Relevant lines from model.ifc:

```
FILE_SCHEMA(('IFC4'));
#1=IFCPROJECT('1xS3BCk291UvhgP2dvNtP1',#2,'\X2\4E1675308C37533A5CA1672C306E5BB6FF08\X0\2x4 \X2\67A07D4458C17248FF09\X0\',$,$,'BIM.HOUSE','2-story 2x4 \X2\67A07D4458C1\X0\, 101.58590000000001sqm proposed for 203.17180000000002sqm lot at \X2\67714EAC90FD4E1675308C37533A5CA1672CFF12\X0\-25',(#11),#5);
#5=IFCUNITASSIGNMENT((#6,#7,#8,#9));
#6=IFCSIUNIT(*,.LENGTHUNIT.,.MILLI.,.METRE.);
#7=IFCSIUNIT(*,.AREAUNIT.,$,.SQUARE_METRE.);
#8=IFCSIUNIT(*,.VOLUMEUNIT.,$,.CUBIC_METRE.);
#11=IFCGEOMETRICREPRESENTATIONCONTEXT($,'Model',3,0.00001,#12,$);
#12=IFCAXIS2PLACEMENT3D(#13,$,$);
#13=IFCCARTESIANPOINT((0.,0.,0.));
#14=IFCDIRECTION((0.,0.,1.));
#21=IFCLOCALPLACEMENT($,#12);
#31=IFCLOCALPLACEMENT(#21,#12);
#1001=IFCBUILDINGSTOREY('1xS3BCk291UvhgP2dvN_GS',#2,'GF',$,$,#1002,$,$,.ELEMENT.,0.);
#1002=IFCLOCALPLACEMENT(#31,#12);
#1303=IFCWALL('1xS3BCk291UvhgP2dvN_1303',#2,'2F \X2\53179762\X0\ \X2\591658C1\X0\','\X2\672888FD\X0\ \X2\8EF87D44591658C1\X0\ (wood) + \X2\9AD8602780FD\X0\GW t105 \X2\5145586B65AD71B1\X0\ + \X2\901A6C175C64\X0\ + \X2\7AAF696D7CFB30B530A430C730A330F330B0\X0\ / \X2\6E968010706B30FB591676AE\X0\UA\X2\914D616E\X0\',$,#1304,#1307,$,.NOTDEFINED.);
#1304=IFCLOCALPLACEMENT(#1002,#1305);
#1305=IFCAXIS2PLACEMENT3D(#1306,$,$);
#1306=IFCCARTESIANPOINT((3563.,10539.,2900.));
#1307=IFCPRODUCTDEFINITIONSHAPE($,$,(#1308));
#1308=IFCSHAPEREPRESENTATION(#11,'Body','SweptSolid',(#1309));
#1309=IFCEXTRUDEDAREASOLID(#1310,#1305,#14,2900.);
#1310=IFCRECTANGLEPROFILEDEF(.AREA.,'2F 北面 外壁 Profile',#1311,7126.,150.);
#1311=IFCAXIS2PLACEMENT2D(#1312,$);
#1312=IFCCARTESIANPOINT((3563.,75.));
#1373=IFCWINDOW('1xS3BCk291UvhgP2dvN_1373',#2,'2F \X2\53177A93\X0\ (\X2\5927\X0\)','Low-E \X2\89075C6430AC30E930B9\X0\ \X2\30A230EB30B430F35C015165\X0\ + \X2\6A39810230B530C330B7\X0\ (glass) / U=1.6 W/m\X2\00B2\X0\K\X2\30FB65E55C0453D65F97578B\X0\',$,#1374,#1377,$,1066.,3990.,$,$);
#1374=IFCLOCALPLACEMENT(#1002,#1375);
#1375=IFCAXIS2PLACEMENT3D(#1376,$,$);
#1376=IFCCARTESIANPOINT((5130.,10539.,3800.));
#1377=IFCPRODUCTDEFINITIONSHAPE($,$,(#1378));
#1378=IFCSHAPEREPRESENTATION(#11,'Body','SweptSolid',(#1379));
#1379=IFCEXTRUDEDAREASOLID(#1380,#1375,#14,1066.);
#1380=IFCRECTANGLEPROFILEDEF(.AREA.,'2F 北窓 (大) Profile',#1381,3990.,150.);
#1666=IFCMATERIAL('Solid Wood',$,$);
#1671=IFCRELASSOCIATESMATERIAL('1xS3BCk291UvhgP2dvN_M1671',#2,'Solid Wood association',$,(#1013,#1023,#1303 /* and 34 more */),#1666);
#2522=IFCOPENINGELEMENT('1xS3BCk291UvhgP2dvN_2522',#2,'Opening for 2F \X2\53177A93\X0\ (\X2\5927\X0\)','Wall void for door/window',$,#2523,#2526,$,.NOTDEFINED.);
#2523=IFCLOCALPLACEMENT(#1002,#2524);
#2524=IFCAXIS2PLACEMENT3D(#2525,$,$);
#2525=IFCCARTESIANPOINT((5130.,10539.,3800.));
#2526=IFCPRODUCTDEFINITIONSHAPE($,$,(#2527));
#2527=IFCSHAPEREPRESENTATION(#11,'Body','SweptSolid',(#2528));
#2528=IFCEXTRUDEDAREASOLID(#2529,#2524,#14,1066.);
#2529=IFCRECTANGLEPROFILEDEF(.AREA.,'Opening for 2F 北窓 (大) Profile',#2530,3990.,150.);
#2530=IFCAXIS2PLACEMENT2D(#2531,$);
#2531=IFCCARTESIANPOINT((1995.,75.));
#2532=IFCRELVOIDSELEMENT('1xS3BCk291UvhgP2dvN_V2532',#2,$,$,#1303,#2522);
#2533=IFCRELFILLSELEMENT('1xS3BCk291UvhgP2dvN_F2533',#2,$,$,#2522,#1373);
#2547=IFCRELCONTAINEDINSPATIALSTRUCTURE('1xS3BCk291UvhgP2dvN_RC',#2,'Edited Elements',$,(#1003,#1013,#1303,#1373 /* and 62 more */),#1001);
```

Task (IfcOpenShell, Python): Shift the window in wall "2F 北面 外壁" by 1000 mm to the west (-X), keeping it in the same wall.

```python
import ifcopenshell
import ifcopenshell.api.geometry
import ifcopenshell.util.placement

model = ifcopenshell.open("model.ifc")

window = model.by_guid("1xS3BCk291UvhgP2dvN_1373")
opening = window.FillsVoids[0].RelatingOpeningElement
wall = opening.VoidsElements[0].RelatingBuildingElement

wall_matrix = ifcopenshell.util.placement.get_local_placement(wall.ObjectPlacement)
shift = wall_matrix[:3, 0] * -1000.0
before = ifcopenshell.util.placement.get_local_placement(window.ObjectPlacement)[:3, 3].copy()

# The window is not placed relative to its opening, so move both.
for product in (opening, window):
    matrix = ifcopenshell.util.placement.get_local_placement(product.ObjectPlacement)
    matrix[:3, 3] += shift
    ifcopenshell.api.geometry.edit_object_placement(model, product=product, matrix=matrix, is_si=False)

after = ifcopenshell.util.placement.get_local_placement(window.ObjectPlacement)[:3, 3]
print("window moved by", (after - before).round(3) + 0.0)

model.write("model_rev.ifc")
```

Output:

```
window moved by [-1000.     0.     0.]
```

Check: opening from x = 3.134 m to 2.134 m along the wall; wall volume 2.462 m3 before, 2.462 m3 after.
